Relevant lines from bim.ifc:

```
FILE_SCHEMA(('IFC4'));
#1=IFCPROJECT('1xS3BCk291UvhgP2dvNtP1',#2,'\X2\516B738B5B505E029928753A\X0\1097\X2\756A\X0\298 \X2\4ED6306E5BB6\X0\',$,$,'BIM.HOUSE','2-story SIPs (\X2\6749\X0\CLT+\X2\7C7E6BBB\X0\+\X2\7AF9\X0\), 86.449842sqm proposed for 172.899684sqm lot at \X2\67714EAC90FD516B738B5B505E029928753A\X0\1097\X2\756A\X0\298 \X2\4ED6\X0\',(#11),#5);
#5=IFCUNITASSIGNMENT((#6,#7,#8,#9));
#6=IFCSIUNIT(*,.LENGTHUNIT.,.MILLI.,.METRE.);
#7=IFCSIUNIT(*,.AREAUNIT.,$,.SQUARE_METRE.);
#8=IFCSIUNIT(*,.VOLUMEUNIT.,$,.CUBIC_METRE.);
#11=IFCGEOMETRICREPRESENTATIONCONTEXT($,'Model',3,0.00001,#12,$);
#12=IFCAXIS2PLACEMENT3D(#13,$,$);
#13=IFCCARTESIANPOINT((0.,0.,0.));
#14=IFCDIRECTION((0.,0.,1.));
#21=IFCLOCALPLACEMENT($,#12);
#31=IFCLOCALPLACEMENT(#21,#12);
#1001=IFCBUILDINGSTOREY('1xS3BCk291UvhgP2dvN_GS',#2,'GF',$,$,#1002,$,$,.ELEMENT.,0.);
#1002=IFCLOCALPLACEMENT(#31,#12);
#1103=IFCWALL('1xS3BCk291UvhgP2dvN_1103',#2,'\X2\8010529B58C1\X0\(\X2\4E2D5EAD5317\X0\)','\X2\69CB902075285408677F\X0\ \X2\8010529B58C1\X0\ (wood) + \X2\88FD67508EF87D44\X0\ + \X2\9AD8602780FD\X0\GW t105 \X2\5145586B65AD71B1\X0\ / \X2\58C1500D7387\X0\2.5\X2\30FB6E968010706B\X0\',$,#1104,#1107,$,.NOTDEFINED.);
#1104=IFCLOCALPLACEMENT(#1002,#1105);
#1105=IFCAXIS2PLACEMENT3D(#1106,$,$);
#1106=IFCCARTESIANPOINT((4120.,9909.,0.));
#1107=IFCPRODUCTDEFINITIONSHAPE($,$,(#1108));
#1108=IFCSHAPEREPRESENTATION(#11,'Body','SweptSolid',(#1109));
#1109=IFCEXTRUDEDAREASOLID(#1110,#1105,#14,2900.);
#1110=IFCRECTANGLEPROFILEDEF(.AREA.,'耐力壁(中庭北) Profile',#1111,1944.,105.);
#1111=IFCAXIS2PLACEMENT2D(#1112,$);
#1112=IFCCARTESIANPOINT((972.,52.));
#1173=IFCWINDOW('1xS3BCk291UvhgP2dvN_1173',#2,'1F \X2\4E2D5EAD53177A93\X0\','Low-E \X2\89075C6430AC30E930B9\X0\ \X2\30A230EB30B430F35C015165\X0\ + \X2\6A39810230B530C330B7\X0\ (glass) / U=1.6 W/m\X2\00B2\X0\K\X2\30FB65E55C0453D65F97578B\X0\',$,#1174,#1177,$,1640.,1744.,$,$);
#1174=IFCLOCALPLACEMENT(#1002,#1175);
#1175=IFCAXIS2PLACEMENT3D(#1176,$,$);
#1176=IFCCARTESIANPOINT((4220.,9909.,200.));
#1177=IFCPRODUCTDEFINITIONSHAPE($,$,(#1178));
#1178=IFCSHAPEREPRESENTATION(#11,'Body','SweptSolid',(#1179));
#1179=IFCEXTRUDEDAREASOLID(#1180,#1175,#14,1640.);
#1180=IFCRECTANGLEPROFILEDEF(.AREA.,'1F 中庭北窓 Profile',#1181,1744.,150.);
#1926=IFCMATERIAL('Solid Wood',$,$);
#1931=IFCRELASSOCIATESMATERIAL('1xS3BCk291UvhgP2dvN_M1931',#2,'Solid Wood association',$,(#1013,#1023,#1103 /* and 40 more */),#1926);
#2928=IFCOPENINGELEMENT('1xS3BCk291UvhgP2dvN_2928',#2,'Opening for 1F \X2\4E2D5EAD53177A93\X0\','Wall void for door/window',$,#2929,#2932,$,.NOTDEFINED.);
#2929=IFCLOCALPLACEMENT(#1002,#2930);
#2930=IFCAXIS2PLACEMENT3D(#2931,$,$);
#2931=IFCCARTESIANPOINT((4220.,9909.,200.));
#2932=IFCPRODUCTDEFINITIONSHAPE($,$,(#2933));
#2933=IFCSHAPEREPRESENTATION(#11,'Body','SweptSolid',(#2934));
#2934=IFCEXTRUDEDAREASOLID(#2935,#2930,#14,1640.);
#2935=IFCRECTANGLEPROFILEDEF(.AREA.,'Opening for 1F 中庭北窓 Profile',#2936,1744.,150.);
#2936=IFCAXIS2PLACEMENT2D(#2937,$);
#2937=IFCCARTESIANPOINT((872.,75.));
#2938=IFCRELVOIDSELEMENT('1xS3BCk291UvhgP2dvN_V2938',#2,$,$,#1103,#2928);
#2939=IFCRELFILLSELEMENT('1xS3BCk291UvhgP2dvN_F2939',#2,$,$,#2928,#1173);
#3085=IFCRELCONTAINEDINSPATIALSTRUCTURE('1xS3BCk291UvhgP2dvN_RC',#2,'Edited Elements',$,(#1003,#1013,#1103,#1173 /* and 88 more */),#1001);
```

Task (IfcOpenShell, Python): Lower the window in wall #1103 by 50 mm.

```python
import numpy as np
import ifcopenshell
import ifcopenshell.api.geometry
import ifcopenshell.util.placement
import ifcopenshell.util.unit

model = ifcopenshell.open("bim.ifc")
unit_scale = ifcopenshell.util.unit.calculate_unit_scale(model)

window = model.by_guid("1xS3BCk291UvhgP2dvN_1173")
opening = window.FillsVoids[0].RelatingOpeningElement
dz = -0.05 / unit_scale

shift = np.array([0.0, 0.0, dz])
# The window is not placed relative to its opening, so move both.
for product in (opening, window):
    matrix = ifcopenshell.util.placement.get_local_placement(product.ObjectPlacement)
    matrix[:3, 3] += shift
    ifcopenshell.api.geometry.edit_object_placement(model, product=product, matrix=matrix, is_si=False)

print(f"moved by {dz * unit_scale:+.3f} m")

model.write("bim-out.ifc")
```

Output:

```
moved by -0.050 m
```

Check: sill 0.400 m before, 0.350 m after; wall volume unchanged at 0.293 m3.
